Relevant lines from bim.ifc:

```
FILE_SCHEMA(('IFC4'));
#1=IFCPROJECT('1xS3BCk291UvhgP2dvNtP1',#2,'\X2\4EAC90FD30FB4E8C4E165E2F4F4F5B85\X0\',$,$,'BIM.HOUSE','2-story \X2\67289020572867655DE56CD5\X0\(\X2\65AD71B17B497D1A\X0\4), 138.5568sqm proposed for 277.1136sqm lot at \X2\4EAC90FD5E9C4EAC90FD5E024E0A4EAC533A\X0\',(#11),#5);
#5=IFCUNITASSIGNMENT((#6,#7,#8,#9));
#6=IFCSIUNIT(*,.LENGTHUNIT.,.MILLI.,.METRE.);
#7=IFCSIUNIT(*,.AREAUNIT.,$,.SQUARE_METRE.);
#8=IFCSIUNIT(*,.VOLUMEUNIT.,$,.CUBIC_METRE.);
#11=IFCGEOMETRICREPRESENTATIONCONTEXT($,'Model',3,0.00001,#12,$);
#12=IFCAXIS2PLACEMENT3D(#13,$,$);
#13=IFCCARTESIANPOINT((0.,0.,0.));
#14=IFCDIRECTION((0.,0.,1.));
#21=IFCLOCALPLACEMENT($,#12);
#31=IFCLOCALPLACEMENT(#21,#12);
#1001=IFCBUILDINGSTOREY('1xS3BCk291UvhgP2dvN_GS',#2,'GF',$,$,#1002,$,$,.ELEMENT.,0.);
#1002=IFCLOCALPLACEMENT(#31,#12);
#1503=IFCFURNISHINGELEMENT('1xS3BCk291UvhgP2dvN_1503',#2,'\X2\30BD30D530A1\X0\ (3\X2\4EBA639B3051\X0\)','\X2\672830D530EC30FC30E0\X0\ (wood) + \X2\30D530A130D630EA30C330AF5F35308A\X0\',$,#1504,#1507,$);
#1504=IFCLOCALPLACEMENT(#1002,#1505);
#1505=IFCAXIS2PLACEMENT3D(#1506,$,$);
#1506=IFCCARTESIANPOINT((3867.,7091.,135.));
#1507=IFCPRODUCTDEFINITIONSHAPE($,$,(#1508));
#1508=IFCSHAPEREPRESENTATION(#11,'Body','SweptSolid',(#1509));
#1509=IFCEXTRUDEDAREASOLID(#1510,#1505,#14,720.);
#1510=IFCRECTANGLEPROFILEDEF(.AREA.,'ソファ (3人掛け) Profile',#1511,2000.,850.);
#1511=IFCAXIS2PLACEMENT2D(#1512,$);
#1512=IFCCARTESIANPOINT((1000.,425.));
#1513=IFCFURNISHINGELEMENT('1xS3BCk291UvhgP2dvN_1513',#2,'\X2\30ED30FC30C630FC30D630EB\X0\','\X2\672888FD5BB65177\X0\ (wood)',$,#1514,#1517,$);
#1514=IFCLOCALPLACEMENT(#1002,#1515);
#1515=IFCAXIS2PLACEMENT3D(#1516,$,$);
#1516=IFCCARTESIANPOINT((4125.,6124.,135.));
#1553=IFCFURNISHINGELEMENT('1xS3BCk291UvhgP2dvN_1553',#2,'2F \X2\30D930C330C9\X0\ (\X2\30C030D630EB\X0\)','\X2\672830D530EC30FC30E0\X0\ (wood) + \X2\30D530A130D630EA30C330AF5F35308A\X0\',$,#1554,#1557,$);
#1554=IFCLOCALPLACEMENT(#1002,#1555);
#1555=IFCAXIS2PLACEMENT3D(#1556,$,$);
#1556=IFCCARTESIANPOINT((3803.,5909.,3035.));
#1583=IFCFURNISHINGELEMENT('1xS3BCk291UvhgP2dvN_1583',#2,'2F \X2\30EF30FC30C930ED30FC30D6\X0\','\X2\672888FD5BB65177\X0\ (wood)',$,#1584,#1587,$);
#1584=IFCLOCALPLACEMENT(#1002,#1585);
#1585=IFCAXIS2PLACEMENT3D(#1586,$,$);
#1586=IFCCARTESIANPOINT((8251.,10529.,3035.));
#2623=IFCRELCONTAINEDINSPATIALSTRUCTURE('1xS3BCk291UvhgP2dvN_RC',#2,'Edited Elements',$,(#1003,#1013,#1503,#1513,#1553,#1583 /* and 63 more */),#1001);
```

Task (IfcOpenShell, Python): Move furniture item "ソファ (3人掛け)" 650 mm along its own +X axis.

```python
import ifcopenshell
import ifcopenshell.api.geometry
import ifcopenshell.util.placement

model = ifcopenshell.open("bim.ifc")

item = model.by_guid("1xS3BCk291UvhgP2dvN_1503")
matrix = ifcopenshell.util.placement.get_local_placement(item.ObjectPlacement)
matrix[:3, 3] += matrix[:3, 0] * 650.0
ifcopenshell.api.geometry.edit_object_placement(model, product=item, matrix=matrix, is_si=False)

print(ifcopenshell.util.placement.get_local_placement(item.ObjectPlacement).round(3) + 0.0)

model.write("bim_edited.ifc")
```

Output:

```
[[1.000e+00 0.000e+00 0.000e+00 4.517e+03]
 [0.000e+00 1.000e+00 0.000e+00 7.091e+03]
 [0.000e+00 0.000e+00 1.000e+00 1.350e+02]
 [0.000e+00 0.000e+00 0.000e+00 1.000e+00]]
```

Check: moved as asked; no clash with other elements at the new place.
